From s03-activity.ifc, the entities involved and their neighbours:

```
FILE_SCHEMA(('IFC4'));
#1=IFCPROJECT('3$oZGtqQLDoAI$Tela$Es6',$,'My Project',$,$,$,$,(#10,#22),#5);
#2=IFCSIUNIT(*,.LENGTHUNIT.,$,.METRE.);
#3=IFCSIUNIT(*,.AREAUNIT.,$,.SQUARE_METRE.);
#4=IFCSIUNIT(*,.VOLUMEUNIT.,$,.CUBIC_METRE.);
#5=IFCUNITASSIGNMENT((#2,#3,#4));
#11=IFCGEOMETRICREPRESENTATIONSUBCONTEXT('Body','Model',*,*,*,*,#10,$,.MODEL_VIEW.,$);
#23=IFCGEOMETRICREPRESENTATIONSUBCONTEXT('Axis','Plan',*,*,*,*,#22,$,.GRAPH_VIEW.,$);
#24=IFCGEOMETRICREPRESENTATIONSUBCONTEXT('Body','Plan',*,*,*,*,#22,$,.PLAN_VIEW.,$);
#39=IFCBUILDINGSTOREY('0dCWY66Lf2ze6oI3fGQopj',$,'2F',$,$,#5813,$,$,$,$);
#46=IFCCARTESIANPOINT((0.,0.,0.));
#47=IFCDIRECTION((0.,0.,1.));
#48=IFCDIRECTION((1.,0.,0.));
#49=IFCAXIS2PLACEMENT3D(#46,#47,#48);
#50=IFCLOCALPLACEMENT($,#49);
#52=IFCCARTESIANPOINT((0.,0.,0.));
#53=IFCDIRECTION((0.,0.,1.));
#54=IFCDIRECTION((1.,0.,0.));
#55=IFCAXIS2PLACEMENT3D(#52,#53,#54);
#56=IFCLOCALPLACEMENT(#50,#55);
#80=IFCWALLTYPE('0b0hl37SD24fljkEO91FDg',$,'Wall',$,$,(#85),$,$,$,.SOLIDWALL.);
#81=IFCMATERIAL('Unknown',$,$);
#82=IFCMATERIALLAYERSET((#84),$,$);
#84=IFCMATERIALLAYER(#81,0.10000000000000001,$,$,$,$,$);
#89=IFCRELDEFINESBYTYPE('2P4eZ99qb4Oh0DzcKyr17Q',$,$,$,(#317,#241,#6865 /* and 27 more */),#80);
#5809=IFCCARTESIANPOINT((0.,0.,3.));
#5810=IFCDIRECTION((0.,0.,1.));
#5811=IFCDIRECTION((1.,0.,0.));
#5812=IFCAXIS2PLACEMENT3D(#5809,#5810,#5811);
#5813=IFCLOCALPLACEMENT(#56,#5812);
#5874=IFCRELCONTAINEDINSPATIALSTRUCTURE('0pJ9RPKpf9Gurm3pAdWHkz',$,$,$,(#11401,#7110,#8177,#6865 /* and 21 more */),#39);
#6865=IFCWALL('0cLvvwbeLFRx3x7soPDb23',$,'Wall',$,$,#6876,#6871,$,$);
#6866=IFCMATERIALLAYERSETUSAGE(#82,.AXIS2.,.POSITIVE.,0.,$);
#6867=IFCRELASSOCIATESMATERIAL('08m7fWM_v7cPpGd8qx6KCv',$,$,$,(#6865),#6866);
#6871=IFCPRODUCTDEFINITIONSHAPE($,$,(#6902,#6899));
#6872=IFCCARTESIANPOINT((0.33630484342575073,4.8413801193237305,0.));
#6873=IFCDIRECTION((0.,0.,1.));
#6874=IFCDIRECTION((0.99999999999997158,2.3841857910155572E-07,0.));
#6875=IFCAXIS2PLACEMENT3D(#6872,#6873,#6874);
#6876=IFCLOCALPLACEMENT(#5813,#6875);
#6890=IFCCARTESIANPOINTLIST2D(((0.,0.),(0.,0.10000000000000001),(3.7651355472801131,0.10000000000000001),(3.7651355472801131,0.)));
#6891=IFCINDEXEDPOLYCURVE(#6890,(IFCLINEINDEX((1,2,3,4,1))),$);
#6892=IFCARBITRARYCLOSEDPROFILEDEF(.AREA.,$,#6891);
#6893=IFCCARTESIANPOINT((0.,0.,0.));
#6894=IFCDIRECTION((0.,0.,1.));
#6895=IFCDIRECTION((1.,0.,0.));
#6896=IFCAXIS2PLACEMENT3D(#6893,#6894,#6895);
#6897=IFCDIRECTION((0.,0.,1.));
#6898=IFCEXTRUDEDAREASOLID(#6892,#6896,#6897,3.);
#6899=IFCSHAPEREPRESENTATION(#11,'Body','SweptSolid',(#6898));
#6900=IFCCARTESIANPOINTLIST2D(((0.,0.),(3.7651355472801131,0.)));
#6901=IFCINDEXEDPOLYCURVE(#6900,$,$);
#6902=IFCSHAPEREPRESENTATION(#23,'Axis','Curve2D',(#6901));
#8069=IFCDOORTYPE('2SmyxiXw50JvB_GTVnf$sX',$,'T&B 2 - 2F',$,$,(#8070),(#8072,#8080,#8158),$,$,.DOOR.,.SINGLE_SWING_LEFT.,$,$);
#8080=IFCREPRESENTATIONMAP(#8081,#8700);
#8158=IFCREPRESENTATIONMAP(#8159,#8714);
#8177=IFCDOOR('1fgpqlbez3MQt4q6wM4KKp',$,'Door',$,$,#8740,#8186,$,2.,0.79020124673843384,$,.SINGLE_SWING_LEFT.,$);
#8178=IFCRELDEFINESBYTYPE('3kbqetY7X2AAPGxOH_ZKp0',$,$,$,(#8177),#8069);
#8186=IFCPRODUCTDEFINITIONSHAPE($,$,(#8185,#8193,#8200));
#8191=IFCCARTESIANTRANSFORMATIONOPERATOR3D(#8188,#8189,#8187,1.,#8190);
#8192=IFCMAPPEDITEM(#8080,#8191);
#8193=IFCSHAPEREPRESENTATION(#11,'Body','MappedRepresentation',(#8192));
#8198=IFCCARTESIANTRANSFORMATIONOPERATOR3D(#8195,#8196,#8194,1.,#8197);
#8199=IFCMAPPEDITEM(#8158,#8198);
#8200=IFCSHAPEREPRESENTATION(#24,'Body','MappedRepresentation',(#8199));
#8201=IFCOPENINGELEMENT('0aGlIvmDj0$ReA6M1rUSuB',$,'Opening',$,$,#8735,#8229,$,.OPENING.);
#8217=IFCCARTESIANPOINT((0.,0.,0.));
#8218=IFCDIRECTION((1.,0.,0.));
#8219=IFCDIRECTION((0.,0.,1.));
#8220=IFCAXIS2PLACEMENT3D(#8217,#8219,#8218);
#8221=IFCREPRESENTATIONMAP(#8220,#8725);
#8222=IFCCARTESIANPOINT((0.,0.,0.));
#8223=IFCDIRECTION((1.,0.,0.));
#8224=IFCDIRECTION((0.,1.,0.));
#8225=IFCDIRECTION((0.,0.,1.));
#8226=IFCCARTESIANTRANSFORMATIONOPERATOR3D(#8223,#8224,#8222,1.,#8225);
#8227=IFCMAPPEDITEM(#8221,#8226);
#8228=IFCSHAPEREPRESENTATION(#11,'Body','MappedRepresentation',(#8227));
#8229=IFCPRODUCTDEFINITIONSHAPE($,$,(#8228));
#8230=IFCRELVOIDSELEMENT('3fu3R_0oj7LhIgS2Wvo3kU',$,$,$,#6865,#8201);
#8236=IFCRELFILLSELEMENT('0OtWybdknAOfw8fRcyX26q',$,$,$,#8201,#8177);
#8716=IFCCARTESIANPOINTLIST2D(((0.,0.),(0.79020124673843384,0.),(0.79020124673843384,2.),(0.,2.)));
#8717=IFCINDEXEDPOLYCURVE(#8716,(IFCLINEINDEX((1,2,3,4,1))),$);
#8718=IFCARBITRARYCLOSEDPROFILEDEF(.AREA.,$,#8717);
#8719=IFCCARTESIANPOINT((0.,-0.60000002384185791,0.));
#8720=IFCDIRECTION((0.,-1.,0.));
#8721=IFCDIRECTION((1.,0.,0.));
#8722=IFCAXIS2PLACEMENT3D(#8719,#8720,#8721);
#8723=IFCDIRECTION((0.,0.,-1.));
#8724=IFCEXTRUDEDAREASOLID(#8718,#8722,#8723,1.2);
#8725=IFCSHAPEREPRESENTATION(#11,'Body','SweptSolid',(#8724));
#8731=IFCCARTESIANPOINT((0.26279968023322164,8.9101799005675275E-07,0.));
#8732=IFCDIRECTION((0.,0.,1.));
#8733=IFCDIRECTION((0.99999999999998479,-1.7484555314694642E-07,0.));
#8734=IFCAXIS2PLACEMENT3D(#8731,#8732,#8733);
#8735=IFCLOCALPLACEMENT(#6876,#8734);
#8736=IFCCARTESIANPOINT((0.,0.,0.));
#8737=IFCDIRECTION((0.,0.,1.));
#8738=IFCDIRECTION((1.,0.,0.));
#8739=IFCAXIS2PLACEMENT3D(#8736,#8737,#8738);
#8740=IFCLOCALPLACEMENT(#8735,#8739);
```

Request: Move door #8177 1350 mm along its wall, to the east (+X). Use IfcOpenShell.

```python
import ifcopenshell
import ifcopenshell.api.geometry
import ifcopenshell.util.placement
import ifcopenshell.util.unit

model = ifcopenshell.open("s03-activity.ifc")
unit_scale = ifcopenshell.util.unit.calculate_unit_scale(model)

door = model.by_guid("1fgpqlbez3MQt4q6wM4KKp")
opening = door.FillsVoids[0].RelatingOpeningElement
wall = opening.VoidsElements[0].RelatingBuildingElement

wall_matrix = ifcopenshell.util.placement.get_local_placement(wall.ObjectPlacement)
shift = wall_matrix[:3, 0] * 1.35 / unit_scale
before = ifcopenshell.util.placement.get_local_placement(door.ObjectPlacement)[:3, 3].copy()

# The door is placed relative to its opening, so it follows when the opening moves.
matrix = ifcopenshell.util.placement.get_local_placement(opening.ObjectPlacement)
matrix[:3, 3] += shift
ifcopenshell.api.geometry.edit_object_placement(
    model, product=opening, matrix=matrix, is_si=False, should_transform_children=True
)

after = ifcopenshell.util.placement.get_local_placement(door.ObjectPlacement)[:3, 3]
print("door moved by", (after - before).round(3) + 0.0)

model.write("s03-activity-out.ifc")
```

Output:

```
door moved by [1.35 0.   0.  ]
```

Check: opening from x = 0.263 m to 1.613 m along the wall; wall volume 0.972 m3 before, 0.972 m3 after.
